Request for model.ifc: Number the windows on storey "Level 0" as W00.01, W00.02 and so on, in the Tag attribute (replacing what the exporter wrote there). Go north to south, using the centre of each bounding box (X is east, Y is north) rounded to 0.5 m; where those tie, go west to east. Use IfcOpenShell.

First a look at what the model holds.

```python
import ifcopenshell
import ifcopenshell.util.element
import ifcopenshell.util.placement

model = ifcopenshell.open("model.ifc")
print(model.schema)
storey = next(s for s in model.by_type("IfcBuildingStorey") if s.Name == "Level 0")
windows = [e for e in ifcopenshell.util.element.get_decomposition(storey) if e.is_a("IfcWindow")]
for e in sorted(windows, key=lambda e: e.id()):
    origin = ifcopenshell.util.placement.get_local_placement(e.ObjectPlacement)[:3, 3]
    print(e.id(), e.Tag, e.Name, origin.round(2) + 0.0, sep=" | ")
```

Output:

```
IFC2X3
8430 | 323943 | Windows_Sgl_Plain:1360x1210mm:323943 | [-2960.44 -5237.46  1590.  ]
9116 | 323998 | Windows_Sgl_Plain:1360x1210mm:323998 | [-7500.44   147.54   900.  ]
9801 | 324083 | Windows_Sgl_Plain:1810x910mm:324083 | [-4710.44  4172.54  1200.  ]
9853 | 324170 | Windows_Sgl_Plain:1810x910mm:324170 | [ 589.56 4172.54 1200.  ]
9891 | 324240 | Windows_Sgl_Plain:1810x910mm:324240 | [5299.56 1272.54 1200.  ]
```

```python
import ifcopenshell
import ifcopenshell.geom
import ifcopenshell.util.element
import ifcopenshell.util.shape

model = ifcopenshell.open("model.ifc")
settings = ifcopenshell.geom.settings()
settings.set("use-world-coords", True)


def centre(element):
    shape = ifcopenshell.geom.create_shape(settings, element)
    return ifcopenshell.util.shape.get_bbox_centroid(shape.geometry)


storey = next(s for s in model.by_type("IfcBuildingStorey") if s.Name == "Level 0")
windows = [e for e in ifcopenshell.util.element.get_decomposition(storey) if e.is_a("IfcWindow")]

# Insertion points can sit at a corner or the storey origin, so sort by the geometry (in metres).
centres = {e: centre(e) for e in windows}
windows.sort(key=lambda e: (-round(centres[e][1] / 0.5), centres[e][0]))

for i, e in enumerate(windows, start=1):
    number = f"W00.{i:02d}"
    e.Tag = number
    print(e.id(), number)

model.write("model_v2.ifc")
```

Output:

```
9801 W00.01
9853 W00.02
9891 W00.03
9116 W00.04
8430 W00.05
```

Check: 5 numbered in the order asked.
